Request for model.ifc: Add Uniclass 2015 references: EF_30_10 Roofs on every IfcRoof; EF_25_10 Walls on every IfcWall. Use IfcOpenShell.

First a look at what the model holds.

```python
import ifcopenshell

model = ifcopenshell.open("model.ifc")
print(model.schema)
print("classifications:", [c.Name for c in model.by_type("IfcClassification")])
for ifc_class in ("IfcDoor", "IfcRoof", "IfcStair", "IfcWall", "IfcWindow"):
    print(ifc_class, len(model.by_type(ifc_class)))
```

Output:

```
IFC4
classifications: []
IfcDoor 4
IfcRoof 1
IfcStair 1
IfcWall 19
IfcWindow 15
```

```python
import ifcopenshell
import ifcopenshell.api.classification

model = ifcopenshell.open("model.ifc")

system = ifcopenshell.api.classification.add_classification(model, classification="Uniclass 2015")

codes = {
    "IfcRoof": ("EF_30_10", "Roofs"),
    "IfcWall": ("EF_25_10", "Walls"),
}
for ifc_class, (code, name) in codes.items():
    products = model.by_type(ifc_class)
    ifcopenshell.api.classification.add_reference(
        model, products=products, classification=system, identification=code, name=name
    )
    print(code, len(products))

model.write("model_edited.ifc")
```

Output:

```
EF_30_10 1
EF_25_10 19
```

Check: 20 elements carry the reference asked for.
